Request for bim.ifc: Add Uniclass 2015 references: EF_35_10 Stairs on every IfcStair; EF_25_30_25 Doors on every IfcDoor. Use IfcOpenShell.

First a look at what the model holds.

```python
import ifcopenshell

model = ifcopenshell.open("bim.ifc")
print(model.schema)
print("classifications:", [c.Name for c in model.by_type("IfcClassification")])
for ifc_class in ("IfcDoor", "IfcRoof", "IfcStair", "IfcWall", "IfcWindow"):
    print(ifc_class, len(model.by_type(ifc_class)))
```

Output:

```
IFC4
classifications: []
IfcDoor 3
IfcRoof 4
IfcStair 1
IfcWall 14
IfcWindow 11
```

```python
import ifcopenshell
import ifcopenshell.api.classification

model = ifcopenshell.open("bim.ifc")

system = ifcopenshell.api.classification.add_classification(model, classification="Uniclass 2015")

codes = {
    "IfcStair": ("EF_35_10", "Stairs"),
    "IfcDoor": ("EF_25_30_25", "Doors"),
}
for ifc_class, (code, name) in codes.items():
    products = model.by_type(ifc_class)
    ifcopenshell.api.classification.add_reference(
        model, products=products, classification=system, identification=code, name=name
    )
    print(code, len(products))

model.write("bim-out.ifc")
```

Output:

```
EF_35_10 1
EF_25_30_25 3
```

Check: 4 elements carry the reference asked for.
